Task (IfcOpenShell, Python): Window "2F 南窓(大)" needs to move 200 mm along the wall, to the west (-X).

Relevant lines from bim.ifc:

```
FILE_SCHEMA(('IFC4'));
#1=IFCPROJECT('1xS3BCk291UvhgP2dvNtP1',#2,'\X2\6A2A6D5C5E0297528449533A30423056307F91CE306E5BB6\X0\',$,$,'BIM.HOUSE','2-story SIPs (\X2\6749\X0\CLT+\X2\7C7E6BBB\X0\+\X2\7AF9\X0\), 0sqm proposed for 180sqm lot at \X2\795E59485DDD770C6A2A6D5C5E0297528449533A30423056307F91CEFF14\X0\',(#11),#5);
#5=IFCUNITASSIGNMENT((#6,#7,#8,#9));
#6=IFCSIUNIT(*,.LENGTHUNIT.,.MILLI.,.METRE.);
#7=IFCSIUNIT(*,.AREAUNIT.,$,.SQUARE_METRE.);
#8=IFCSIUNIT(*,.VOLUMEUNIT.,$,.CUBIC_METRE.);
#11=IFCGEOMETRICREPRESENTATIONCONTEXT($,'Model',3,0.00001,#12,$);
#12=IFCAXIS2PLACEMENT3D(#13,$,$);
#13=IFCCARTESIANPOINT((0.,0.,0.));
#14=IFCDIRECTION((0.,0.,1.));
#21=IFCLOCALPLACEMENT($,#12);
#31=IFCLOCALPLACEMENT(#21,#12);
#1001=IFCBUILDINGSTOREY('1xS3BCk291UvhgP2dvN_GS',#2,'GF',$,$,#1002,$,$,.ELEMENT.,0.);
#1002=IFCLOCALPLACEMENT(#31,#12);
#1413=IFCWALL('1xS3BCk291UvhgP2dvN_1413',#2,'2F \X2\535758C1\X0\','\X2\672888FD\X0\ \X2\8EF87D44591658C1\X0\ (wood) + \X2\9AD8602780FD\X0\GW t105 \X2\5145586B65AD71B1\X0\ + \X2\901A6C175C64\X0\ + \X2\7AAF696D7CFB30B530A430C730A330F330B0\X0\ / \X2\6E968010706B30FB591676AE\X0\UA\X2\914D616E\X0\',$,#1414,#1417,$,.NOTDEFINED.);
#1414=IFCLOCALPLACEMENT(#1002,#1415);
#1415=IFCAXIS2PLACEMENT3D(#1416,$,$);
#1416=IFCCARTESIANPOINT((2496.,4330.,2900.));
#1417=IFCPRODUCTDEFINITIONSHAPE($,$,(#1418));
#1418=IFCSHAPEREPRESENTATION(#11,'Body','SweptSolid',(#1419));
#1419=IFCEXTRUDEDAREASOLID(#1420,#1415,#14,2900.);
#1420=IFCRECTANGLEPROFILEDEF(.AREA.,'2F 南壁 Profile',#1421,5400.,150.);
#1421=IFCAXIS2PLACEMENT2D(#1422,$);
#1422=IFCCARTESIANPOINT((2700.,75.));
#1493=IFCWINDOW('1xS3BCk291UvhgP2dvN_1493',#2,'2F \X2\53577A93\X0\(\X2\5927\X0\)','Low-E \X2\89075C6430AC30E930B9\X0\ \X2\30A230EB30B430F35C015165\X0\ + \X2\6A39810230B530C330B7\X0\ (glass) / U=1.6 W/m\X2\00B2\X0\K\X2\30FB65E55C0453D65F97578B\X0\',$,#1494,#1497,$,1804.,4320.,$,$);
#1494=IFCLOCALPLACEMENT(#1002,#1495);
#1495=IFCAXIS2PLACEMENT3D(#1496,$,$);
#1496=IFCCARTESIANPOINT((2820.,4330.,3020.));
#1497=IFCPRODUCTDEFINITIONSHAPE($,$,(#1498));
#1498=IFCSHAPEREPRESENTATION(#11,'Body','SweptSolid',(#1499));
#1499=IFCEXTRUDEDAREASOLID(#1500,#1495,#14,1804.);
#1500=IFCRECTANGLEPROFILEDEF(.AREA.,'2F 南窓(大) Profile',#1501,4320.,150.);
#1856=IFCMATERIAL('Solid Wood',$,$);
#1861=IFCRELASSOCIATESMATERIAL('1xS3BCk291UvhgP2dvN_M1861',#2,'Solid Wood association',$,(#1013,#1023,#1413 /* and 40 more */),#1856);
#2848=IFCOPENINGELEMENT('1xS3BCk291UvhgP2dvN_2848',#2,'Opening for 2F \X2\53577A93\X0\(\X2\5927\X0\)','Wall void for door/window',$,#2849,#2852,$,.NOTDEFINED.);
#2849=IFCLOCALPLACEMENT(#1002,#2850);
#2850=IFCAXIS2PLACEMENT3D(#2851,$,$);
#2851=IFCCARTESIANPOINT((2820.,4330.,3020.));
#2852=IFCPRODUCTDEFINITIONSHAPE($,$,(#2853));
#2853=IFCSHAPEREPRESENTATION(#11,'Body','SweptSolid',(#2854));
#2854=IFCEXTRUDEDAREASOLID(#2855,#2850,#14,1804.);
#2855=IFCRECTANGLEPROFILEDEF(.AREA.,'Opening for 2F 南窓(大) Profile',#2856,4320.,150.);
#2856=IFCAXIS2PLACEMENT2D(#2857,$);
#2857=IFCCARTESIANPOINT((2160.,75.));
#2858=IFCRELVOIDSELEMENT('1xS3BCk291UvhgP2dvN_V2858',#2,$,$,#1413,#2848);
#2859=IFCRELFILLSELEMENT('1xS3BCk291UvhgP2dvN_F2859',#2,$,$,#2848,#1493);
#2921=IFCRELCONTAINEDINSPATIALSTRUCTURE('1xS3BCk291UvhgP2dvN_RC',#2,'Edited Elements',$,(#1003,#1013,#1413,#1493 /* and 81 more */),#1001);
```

```python
import ifcopenshell
import ifcopenshell.api.geometry
import ifcopenshell.util.placement

model = ifcopenshell.open("bim.ifc")

window = model.by_id(1493)
opening = window.FillsVoids[0].RelatingOpeningElement
wall = opening.VoidsElements[0].RelatingBuildingElement

wall_matrix = ifcopenshell.util.placement.get_local_placement(wall.ObjectPlacement)
shift = wall_matrix[:3, 0] * -200.0
before = ifcopenshell.util.placement.get_local_placement(window.ObjectPlacement)[:3, 3].copy()

# The window is not placed relative to its opening, so move both.
for product in (opening, window):
    matrix = ifcopenshell.util.placement.get_local_placement(product.ObjectPlacement)
    matrix[:3, 3] += shift
    ifcopenshell.api.geometry.edit_object_placement(model, product=product, matrix=matrix, is_si=False)

after = ifcopenshell.util.placement.get_local_placement(window.ObjectPlacement)[:3, 3]
print("window moved by", (after - before).round(3) + 0.0)

model.write("bim_v2.ifc")
```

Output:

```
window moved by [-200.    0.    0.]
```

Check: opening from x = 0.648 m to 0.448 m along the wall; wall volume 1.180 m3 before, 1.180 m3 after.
